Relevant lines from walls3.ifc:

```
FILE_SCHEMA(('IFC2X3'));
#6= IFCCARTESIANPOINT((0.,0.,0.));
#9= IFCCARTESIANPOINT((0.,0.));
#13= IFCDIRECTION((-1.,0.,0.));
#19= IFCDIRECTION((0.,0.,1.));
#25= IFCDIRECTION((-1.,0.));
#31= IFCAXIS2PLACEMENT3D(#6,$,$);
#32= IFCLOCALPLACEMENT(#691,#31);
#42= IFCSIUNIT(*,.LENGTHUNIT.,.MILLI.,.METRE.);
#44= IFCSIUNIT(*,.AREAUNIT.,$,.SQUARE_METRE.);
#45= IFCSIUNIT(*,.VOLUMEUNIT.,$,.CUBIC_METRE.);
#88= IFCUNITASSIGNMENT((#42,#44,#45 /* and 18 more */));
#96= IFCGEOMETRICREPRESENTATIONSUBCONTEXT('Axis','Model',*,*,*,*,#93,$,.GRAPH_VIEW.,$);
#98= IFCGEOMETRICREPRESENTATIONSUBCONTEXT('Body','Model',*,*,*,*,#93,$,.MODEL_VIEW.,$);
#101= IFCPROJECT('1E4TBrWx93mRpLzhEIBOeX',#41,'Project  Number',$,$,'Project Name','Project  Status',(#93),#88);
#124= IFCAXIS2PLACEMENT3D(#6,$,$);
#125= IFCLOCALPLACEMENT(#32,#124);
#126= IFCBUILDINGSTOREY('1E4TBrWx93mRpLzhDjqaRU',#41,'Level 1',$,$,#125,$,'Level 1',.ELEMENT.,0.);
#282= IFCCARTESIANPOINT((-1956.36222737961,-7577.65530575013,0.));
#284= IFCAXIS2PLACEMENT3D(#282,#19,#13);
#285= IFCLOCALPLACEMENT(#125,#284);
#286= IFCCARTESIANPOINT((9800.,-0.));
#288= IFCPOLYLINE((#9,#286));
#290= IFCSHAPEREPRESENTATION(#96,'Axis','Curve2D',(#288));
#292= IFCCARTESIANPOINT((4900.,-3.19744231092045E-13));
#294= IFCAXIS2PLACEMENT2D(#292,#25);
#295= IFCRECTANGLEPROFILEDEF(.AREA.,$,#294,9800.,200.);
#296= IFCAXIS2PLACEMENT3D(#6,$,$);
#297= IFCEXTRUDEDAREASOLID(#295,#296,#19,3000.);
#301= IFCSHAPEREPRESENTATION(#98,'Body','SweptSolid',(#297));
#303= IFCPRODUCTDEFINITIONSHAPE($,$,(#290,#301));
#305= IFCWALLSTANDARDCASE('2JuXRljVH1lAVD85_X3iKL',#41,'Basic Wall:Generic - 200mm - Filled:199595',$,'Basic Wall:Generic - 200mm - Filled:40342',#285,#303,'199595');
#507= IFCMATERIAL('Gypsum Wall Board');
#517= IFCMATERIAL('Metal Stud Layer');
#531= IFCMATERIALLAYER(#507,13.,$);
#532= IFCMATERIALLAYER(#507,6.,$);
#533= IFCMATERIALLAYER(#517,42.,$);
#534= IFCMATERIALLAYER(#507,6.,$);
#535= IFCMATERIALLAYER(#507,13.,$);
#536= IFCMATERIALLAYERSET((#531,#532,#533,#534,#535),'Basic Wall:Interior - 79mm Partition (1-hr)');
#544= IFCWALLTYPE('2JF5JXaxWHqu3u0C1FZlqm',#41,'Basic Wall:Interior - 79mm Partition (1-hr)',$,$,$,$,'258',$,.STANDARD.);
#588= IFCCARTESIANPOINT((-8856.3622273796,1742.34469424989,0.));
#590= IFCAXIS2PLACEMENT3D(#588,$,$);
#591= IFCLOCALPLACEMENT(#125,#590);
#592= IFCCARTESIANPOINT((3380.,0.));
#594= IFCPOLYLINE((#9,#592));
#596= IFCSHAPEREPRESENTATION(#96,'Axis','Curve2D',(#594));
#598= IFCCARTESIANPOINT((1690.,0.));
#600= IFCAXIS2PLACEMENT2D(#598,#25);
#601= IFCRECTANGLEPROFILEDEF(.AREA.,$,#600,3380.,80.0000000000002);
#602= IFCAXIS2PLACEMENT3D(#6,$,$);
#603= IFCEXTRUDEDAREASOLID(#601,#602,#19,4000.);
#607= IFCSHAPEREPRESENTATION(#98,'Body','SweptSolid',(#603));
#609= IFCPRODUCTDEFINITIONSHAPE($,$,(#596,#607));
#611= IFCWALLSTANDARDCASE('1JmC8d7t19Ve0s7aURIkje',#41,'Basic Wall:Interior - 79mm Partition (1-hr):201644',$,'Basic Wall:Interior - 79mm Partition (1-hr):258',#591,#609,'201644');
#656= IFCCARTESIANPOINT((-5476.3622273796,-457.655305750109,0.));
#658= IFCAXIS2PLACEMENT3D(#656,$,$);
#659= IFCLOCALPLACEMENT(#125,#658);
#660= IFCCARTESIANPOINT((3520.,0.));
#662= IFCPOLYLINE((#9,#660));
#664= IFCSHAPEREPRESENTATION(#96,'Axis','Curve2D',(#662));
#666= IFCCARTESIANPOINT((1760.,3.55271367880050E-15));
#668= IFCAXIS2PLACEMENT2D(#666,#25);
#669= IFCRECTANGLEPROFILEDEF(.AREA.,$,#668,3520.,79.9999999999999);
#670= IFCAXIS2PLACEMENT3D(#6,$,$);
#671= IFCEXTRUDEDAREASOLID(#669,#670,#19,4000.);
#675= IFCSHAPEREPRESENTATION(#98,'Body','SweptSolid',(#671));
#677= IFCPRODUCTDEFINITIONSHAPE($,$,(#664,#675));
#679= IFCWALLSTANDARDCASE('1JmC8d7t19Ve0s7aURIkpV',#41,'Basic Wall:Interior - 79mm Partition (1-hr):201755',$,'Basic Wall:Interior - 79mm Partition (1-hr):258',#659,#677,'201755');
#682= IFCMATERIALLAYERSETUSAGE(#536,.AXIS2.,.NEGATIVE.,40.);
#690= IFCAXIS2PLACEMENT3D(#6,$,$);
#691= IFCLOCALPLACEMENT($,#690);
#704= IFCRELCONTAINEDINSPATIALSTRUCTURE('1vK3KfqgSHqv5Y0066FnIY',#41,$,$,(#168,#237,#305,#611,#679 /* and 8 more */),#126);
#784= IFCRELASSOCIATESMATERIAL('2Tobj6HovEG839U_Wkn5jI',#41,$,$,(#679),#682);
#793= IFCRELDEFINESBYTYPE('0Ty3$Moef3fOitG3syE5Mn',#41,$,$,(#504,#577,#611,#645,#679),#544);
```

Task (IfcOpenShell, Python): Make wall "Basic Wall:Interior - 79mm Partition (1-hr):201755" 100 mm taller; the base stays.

```python
import ifcopenshell
import ifcopenshell.geom
import ifcopenshell.util.representation
import ifcopenshell.util.shape
import ifcopenshell.util.unit

model = ifcopenshell.open("walls3.ifc")
unit_scale = ifcopenshell.util.unit.calculate_unit_scale(model)
settings = ifcopenshell.geom.settings()


def volume(element):
    """Net volume in cubic metres, openings subtracted."""
    shape = ifcopenshell.geom.create_shape(settings, element)
    return ifcopenshell.util.shape.get_volume(shape.geometry)


wall = model.by_guid("1JmC8d7t19Ve0s7aURIkpV")
before = volume(wall)

body = ifcopenshell.util.representation.get_representation(wall, "Model", "Body")
solid = body.Items[0]
old_height = solid.Depth
solid.Depth += 0.1 / unit_scale
after = volume(wall)

print(f"height {old_height:g} -> {solid.Depth:g}, volume {before:.3f} -> {after:.3f} m3")

model.write("walls3_v2.ifc")
```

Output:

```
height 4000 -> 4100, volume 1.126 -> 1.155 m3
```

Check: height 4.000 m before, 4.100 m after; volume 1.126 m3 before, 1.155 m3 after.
